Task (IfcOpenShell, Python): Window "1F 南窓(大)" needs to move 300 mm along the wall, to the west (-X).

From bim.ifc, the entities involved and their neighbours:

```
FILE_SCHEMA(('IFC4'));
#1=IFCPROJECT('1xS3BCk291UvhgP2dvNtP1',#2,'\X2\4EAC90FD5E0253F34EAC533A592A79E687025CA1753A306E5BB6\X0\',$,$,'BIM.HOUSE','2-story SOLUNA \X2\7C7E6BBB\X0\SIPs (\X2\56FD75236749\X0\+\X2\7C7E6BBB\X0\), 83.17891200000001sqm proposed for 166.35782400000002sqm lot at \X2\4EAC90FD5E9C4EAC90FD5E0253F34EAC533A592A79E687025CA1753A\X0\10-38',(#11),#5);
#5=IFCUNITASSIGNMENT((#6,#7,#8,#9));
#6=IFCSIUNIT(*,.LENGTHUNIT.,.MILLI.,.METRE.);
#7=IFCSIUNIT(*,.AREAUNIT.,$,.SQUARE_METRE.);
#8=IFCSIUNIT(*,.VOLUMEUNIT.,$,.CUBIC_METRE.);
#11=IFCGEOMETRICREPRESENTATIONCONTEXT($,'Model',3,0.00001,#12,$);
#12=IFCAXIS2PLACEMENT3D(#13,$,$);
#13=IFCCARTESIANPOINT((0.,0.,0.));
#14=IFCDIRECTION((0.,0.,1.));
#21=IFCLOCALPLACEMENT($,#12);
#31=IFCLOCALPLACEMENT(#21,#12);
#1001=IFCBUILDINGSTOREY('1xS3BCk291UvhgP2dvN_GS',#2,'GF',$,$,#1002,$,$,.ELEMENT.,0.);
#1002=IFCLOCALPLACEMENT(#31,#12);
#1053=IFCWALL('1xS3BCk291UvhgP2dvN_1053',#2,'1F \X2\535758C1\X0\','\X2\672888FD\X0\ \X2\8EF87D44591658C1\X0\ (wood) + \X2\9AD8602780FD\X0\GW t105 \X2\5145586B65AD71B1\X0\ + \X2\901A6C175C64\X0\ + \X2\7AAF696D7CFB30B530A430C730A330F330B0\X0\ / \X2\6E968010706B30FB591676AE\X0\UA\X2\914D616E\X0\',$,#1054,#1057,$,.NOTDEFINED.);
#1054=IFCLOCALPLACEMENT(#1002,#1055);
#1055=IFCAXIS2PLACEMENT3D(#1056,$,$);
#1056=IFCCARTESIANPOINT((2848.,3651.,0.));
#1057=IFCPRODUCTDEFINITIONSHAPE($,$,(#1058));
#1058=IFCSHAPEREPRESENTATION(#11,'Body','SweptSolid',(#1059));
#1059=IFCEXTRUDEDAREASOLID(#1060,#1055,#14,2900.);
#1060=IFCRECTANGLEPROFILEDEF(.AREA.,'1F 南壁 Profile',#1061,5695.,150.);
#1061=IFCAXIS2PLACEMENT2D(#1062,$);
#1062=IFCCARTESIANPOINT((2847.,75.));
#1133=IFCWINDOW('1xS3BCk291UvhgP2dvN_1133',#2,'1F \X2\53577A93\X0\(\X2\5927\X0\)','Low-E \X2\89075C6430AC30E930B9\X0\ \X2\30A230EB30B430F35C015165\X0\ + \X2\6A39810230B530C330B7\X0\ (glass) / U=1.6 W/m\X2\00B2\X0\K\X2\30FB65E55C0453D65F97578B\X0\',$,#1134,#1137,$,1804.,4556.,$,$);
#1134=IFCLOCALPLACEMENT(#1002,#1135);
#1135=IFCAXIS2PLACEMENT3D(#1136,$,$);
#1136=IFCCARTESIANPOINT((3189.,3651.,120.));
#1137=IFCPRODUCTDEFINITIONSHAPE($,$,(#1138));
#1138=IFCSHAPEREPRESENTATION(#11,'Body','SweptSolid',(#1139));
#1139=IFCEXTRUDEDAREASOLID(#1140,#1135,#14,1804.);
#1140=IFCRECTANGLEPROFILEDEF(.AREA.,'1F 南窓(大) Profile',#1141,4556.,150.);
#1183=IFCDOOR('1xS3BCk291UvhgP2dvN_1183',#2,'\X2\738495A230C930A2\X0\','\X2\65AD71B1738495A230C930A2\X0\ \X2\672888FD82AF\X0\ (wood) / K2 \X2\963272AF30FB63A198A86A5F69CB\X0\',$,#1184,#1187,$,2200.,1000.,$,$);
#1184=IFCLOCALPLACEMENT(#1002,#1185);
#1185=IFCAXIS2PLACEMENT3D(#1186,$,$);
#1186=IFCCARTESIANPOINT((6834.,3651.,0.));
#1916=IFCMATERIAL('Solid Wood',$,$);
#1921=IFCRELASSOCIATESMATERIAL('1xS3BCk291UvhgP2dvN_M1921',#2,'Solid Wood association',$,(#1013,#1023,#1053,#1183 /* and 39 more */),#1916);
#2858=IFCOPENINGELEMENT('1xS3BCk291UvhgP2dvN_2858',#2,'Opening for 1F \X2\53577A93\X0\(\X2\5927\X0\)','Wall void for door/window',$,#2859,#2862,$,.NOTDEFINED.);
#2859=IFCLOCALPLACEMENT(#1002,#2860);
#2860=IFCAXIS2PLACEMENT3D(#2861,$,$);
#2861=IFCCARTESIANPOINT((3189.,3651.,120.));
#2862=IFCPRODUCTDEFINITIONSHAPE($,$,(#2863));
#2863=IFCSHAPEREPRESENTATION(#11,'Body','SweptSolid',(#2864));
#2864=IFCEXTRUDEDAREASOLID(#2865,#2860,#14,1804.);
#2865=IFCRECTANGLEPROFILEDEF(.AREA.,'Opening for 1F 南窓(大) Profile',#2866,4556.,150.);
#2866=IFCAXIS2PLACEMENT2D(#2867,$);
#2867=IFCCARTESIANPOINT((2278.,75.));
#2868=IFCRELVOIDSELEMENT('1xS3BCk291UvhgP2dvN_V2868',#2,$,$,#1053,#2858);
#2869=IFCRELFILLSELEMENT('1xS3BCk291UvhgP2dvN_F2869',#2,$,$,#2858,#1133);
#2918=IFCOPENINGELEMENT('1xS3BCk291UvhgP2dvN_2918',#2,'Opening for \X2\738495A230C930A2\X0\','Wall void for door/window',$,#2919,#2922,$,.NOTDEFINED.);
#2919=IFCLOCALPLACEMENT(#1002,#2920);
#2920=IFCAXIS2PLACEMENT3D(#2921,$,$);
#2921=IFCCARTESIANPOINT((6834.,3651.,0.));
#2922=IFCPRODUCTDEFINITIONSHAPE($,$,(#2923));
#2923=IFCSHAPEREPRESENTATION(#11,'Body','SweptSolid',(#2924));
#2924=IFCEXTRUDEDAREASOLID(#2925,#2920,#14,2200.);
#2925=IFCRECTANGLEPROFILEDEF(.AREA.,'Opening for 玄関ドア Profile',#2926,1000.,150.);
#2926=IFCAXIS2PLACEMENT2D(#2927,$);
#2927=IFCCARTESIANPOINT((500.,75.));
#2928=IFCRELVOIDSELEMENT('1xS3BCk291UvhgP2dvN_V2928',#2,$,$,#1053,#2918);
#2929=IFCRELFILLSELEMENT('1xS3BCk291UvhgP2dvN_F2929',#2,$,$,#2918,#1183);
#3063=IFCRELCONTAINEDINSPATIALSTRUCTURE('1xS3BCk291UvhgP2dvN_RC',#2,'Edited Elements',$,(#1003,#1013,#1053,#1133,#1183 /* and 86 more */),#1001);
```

```python
import ifcopenshell
import ifcopenshell.api.geometry
import ifcopenshell.util.placement

model = ifcopenshell.open("bim.ifc")

window = model.by_guid("1xS3BCk291UvhgP2dvN_1133")
opening = window.FillsVoids[0].RelatingOpeningElement
wall = opening.VoidsElements[0].RelatingBuildingElement

wall_matrix = ifcopenshell.util.placement.get_local_placement(wall.ObjectPlacement)
shift = wall_matrix[:3, 0] * -300.0
before = ifcopenshell.util.placement.get_local_placement(window.ObjectPlacement)[:3, 3].copy()

# The window is not placed relative to its opening, so move both.
for product in (opening, window):
    matrix = ifcopenshell.util.placement.get_local_placement(product.ObjectPlacement)
    matrix[:3, 3] += shift
    ifcopenshell.api.geometry.edit_object_placement(model, product=product, matrix=matrix, is_si=False)

after = ifcopenshell.util.placement.get_local_placement(window.ObjectPlacement)[:3, 3]
print("window moved by", (after - before).round(3) + 0.0)

model.write("bim-out.ifc")
```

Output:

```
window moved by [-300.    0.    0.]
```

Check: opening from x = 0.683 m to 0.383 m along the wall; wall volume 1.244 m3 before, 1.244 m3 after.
